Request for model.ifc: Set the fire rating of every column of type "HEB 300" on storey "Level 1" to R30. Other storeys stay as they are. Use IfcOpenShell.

First a look at what the model holds.

```python
import ifcopenshell
import ifcopenshell.util.element

model = ifcopenshell.open("model.ifc")
print(model.schema)
storey = next(s for s in model.by_type("IfcBuildingStorey") if s.Name == "Level 1")
columns = [e for e in ifcopenshell.util.element.get_decomposition(storey) if e.is_a("IfcColumn")]
seen = {}
for e in columns:
    element_type = ifcopenshell.util.element.get_type(e)
    key = (element_type.Name if element_type != e and element_type else None, ifcopenshell.util.element.get_pset(e, "Pset_ColumnCommon", "FireRating"))
    seen[key] = seen.get(key, 0) + 1
for (name, value), count in sorted(seen.items(), key=str):
    print(count, "x", name, "|", value)
```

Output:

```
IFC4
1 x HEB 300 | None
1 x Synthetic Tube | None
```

```python
import ifcopenshell
import ifcopenshell.api.pset
import ifcopenshell.util.element

model = ifcopenshell.open("model.ifc")

storey = next(s for s in model.by_type("IfcBuildingStorey") if s.Name == "Level 1")
columns = [e for e in ifcopenshell.util.element.get_decomposition(storey) if e.is_a("IfcColumn")]

count = 0
for e in columns:
    element_type = ifcopenshell.util.element.get_type(e)
    if element_type in (None, e) or element_type.Name != "HEB 300":
        continue
    # add_pset returns the element's existing set when there is one.
    pset = ifcopenshell.api.pset.add_pset(model, product=e, name="Pset_ColumnCommon")
    ifcopenshell.api.pset.edit_pset(model, pset=pset, properties={"FireRating": "R30"})
    count += 1

print(count, "columns updated")

model.write("model-out.ifc")
```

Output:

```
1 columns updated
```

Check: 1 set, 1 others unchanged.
